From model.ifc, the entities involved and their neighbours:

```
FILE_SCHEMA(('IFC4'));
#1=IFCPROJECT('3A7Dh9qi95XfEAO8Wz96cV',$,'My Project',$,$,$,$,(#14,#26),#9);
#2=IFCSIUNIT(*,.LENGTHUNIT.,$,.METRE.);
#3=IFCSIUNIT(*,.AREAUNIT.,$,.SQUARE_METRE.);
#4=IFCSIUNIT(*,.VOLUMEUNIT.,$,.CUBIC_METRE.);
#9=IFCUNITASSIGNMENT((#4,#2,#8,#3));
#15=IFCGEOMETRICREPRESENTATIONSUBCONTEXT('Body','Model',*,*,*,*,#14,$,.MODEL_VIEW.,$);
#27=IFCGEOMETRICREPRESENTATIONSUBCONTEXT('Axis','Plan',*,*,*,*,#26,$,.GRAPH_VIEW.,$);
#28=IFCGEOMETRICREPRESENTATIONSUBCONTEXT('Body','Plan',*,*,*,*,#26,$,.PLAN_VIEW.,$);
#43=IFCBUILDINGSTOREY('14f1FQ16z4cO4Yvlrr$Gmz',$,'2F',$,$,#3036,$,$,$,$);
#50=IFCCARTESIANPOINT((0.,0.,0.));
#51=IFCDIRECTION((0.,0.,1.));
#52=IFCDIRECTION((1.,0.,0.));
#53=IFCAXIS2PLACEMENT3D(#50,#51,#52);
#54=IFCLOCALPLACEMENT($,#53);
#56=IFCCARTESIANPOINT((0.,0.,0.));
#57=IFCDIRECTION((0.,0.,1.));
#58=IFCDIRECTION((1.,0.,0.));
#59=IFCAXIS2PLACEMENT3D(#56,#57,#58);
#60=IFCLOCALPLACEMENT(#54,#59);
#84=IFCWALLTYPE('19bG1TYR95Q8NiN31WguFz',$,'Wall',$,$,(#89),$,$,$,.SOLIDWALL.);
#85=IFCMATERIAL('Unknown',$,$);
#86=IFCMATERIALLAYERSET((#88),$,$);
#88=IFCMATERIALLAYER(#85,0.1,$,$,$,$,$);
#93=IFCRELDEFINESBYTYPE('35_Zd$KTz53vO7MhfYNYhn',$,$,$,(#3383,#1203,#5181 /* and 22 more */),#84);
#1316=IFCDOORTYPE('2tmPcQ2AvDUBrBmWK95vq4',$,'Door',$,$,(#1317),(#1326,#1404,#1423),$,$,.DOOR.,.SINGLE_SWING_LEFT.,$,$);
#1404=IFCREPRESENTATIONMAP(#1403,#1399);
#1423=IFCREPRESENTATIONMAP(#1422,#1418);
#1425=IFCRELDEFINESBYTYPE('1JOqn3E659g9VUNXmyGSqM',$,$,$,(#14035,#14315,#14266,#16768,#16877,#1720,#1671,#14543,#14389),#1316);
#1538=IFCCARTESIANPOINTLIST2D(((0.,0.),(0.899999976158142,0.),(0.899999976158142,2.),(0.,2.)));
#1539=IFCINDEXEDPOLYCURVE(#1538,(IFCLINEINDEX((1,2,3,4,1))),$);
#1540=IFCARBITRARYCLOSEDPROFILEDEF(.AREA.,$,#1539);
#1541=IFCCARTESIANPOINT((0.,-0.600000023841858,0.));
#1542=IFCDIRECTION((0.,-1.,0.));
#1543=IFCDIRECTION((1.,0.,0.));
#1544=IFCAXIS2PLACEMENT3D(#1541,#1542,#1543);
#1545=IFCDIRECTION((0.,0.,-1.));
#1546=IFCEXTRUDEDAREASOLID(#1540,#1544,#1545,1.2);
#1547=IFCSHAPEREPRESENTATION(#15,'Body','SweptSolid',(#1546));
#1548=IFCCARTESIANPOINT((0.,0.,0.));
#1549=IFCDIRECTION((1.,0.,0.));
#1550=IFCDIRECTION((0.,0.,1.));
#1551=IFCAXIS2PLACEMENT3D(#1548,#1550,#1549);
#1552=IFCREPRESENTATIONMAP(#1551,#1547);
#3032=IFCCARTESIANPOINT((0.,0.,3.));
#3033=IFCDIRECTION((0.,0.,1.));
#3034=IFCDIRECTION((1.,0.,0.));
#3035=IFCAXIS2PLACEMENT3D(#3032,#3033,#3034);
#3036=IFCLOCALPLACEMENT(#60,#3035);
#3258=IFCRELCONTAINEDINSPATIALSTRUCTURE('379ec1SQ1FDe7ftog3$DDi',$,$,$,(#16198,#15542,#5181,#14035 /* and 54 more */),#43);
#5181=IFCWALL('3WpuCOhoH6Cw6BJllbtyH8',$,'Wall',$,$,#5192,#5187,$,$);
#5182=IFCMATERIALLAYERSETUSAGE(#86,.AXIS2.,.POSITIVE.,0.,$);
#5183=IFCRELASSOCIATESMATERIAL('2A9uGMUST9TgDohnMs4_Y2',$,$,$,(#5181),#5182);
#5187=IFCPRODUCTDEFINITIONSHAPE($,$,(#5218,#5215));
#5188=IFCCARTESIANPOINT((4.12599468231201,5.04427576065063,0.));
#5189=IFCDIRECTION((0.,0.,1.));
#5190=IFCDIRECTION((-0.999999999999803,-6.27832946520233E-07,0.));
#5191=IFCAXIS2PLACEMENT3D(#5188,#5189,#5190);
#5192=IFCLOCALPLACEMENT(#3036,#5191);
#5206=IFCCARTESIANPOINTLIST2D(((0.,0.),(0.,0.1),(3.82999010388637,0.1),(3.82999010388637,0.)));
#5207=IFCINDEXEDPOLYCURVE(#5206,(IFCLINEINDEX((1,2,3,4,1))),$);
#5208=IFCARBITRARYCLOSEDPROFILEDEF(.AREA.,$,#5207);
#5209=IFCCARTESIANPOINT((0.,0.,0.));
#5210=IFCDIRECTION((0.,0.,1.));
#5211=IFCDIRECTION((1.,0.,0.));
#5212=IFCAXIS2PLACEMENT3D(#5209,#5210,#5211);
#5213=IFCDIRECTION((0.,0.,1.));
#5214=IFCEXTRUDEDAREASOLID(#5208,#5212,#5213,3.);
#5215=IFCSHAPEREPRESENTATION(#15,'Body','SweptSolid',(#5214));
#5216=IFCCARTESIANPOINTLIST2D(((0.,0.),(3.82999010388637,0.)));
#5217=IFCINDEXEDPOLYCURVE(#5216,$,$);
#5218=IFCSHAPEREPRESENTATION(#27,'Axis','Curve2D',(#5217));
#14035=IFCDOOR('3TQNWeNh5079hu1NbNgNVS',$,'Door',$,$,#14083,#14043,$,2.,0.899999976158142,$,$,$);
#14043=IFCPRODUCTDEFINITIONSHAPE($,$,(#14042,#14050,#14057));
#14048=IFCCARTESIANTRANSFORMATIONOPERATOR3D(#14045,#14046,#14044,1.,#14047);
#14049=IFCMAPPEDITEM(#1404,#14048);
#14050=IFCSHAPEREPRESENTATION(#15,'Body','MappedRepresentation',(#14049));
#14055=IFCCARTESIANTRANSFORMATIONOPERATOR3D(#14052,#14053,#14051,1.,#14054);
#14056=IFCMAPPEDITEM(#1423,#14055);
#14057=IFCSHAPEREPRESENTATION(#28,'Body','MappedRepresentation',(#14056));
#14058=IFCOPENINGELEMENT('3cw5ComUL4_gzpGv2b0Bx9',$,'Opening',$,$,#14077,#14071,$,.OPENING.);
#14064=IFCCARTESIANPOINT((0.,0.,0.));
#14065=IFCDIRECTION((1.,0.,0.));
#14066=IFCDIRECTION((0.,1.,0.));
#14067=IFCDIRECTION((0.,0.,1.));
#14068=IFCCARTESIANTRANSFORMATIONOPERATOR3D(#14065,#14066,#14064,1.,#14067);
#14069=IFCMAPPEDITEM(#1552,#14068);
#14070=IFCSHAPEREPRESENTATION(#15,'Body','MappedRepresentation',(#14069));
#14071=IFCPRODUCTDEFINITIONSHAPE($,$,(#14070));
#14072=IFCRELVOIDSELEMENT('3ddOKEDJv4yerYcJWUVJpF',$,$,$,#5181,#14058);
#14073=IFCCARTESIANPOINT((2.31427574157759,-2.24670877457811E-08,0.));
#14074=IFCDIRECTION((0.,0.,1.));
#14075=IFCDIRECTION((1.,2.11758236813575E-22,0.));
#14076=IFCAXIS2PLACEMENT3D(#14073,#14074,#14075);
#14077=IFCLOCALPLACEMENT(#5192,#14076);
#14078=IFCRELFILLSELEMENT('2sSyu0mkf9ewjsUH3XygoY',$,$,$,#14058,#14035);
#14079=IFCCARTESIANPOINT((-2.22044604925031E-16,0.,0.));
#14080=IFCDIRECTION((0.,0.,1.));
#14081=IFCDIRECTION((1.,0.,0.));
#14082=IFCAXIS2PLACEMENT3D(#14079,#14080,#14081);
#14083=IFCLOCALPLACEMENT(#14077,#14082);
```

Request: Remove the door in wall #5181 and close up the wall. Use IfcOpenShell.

```python
import ifcopenshell
import ifcopenshell.api.feature
import ifcopenshell.api.root
import ifcopenshell.geom
import ifcopenshell.util.shape

model = ifcopenshell.open("model.ifc")
settings = ifcopenshell.geom.settings()


def volume(element):
    """Net volume in cubic metres, openings subtracted."""
    shape = ifcopenshell.geom.create_shape(settings, element)
    return ifcopenshell.util.shape.get_volume(shape.geometry)


door = model.by_id(14035)
opening = door.FillsVoids[0].RelatingOpeningElement
wall = opening.VoidsElements[0].RelatingBuildingElement
before = volume(wall)

ifcopenshell.api.root.remove_product(model, product=door)
ifcopenshell.api.feature.remove_feature(model, feature=opening)

after = volume(wall)

print(f"wall volume {before:.3f} -> {after:.3f} m3")

model.write("model_v2.ifc")
```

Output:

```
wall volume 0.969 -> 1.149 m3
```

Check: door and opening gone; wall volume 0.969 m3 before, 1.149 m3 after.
